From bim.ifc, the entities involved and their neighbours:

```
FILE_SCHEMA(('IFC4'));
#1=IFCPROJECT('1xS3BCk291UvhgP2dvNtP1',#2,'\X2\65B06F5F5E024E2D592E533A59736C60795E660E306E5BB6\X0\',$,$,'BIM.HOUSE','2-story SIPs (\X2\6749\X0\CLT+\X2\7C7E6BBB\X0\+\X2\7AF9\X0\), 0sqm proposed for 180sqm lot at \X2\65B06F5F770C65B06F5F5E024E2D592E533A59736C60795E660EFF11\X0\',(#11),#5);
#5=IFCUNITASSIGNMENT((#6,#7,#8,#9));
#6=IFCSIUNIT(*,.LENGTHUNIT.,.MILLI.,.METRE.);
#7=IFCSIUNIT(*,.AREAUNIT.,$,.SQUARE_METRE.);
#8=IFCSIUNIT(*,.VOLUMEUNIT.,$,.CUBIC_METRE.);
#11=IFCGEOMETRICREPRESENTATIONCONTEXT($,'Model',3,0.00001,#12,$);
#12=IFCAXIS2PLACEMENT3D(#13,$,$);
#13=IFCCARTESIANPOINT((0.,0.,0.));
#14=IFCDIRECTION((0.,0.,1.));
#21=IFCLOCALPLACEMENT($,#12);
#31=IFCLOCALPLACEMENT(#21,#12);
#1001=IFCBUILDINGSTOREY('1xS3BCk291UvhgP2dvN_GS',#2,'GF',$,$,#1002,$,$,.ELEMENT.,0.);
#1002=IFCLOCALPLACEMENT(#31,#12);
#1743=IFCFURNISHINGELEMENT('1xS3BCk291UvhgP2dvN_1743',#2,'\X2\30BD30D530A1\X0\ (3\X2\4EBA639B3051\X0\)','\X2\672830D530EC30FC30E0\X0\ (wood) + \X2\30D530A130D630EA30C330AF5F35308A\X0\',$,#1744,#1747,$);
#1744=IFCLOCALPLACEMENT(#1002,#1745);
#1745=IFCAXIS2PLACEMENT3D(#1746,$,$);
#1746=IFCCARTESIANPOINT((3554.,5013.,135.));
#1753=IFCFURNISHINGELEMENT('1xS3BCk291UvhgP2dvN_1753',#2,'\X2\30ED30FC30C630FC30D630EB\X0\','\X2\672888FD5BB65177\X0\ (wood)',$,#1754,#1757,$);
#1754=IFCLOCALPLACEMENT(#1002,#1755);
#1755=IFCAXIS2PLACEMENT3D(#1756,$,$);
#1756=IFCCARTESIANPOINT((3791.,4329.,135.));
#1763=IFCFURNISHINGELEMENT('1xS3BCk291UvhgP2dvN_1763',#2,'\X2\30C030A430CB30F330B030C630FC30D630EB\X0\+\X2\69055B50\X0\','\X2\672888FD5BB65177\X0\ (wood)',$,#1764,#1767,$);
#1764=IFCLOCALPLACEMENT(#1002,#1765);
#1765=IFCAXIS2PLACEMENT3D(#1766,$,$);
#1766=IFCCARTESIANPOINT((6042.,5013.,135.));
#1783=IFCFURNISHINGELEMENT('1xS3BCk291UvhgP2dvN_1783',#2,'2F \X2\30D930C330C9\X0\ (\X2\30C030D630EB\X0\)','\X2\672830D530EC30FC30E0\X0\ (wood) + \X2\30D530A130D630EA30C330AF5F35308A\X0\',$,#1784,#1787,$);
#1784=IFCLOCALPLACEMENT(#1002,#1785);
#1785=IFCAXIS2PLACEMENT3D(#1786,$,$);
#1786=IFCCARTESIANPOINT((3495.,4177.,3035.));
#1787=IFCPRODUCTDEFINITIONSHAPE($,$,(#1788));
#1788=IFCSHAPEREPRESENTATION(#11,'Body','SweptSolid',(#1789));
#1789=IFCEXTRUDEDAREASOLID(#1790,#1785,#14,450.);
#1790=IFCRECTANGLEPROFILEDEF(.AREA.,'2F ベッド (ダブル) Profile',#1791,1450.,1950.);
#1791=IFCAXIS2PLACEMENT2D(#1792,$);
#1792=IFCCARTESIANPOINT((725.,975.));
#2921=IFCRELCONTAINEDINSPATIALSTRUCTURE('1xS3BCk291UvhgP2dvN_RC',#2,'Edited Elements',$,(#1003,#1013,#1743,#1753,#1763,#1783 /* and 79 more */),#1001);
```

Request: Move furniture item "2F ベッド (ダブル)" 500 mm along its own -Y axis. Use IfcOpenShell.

```python
import ifcopenshell
import ifcopenshell.api.geometry
import ifcopenshell.util.placement
import ifcopenshell.util.unit

model = ifcopenshell.open("bim.ifc")
unit_scale = ifcopenshell.util.unit.calculate_unit_scale(model)

item = model.by_guid("1xS3BCk291UvhgP2dvN_1783")
matrix = ifcopenshell.util.placement.get_local_placement(item.ObjectPlacement)
matrix[:3, 3] -= matrix[:3, 1] * 0.5 / unit_scale
ifcopenshell.api.geometry.edit_object_placement(model, product=item, matrix=matrix, is_si=False)

print(ifcopenshell.util.placement.get_local_placement(item.ObjectPlacement).round(3) + 0.0)

model.write("bim_edited.ifc")
```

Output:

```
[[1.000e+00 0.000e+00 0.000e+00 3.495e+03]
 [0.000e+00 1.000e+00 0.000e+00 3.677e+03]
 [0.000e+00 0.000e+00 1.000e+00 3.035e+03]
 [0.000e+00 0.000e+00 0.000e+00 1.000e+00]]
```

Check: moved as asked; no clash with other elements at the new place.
